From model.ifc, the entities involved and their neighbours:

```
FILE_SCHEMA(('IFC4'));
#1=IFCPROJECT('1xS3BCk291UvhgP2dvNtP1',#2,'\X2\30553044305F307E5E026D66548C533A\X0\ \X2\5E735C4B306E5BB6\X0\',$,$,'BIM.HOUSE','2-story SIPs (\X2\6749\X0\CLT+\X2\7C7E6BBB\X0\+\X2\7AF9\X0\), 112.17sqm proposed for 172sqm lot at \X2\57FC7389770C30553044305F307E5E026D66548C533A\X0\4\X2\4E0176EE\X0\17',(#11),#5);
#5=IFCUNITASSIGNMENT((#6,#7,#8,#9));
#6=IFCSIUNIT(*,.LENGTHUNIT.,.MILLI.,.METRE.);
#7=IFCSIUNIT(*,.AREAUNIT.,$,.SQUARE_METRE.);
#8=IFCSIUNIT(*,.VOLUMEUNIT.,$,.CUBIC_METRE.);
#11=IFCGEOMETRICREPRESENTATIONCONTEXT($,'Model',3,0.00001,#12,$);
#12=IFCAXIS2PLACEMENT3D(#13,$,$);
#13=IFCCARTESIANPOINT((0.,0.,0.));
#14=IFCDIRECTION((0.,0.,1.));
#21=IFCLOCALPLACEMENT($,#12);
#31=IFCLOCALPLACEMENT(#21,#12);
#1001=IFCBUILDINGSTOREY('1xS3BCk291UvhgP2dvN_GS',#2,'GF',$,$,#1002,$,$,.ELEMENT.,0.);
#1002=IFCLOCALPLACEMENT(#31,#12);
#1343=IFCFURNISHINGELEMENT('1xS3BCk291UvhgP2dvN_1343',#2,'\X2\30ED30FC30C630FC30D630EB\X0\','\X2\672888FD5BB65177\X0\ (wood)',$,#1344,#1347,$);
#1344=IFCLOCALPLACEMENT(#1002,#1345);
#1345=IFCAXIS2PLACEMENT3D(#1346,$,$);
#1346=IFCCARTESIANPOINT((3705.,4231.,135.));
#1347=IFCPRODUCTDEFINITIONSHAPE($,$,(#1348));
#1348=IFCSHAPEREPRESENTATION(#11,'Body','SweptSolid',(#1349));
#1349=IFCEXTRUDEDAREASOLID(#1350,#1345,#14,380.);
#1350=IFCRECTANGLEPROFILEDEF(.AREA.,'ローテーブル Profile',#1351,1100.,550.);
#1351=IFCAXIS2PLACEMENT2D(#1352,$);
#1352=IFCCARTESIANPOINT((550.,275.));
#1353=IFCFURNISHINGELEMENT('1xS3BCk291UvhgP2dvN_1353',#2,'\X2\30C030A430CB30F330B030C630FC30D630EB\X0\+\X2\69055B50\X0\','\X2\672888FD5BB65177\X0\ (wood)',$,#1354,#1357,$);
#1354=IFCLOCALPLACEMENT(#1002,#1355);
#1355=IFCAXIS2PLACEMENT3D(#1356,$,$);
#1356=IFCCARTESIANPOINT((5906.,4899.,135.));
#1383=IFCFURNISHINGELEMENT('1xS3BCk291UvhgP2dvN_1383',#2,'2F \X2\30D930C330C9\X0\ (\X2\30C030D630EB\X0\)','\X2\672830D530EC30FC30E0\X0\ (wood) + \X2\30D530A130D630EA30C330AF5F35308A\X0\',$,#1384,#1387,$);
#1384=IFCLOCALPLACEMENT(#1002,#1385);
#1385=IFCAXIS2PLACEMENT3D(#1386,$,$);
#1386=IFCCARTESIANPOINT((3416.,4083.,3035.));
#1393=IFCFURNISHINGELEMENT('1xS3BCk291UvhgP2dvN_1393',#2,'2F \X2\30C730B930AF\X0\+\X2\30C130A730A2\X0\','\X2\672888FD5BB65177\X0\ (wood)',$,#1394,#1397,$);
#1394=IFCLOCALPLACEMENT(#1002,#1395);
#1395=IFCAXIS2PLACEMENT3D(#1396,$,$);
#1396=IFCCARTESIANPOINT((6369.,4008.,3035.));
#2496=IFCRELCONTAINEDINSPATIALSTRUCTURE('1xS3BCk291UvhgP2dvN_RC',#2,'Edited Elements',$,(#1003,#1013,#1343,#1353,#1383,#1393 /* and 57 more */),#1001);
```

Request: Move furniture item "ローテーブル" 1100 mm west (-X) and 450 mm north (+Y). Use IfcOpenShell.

```python
import ifcopenshell
import ifcopenshell.api.geometry
import ifcopenshell.util.placement
import ifcopenshell.util.unit

model = ifcopenshell.open("model.ifc")
unit_scale = ifcopenshell.util.unit.calculate_unit_scale(model)

item = model.by_guid("1xS3BCk291UvhgP2dvN_1343")
matrix = ifcopenshell.util.placement.get_local_placement(item.ObjectPlacement)
matrix[0, 3] -= 1.1 / unit_scale
matrix[1, 3] += 0.45 / unit_scale
ifcopenshell.api.geometry.edit_object_placement(model, product=item, matrix=matrix, is_si=False)

print(ifcopenshell.util.placement.get_local_placement(item.ObjectPlacement).round(3) + 0.0)

model.write("model_edited.ifc")
```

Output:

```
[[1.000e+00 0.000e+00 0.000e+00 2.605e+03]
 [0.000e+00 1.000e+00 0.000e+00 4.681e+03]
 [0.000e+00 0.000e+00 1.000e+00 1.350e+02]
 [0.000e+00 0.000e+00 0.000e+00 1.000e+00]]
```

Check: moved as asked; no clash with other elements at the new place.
